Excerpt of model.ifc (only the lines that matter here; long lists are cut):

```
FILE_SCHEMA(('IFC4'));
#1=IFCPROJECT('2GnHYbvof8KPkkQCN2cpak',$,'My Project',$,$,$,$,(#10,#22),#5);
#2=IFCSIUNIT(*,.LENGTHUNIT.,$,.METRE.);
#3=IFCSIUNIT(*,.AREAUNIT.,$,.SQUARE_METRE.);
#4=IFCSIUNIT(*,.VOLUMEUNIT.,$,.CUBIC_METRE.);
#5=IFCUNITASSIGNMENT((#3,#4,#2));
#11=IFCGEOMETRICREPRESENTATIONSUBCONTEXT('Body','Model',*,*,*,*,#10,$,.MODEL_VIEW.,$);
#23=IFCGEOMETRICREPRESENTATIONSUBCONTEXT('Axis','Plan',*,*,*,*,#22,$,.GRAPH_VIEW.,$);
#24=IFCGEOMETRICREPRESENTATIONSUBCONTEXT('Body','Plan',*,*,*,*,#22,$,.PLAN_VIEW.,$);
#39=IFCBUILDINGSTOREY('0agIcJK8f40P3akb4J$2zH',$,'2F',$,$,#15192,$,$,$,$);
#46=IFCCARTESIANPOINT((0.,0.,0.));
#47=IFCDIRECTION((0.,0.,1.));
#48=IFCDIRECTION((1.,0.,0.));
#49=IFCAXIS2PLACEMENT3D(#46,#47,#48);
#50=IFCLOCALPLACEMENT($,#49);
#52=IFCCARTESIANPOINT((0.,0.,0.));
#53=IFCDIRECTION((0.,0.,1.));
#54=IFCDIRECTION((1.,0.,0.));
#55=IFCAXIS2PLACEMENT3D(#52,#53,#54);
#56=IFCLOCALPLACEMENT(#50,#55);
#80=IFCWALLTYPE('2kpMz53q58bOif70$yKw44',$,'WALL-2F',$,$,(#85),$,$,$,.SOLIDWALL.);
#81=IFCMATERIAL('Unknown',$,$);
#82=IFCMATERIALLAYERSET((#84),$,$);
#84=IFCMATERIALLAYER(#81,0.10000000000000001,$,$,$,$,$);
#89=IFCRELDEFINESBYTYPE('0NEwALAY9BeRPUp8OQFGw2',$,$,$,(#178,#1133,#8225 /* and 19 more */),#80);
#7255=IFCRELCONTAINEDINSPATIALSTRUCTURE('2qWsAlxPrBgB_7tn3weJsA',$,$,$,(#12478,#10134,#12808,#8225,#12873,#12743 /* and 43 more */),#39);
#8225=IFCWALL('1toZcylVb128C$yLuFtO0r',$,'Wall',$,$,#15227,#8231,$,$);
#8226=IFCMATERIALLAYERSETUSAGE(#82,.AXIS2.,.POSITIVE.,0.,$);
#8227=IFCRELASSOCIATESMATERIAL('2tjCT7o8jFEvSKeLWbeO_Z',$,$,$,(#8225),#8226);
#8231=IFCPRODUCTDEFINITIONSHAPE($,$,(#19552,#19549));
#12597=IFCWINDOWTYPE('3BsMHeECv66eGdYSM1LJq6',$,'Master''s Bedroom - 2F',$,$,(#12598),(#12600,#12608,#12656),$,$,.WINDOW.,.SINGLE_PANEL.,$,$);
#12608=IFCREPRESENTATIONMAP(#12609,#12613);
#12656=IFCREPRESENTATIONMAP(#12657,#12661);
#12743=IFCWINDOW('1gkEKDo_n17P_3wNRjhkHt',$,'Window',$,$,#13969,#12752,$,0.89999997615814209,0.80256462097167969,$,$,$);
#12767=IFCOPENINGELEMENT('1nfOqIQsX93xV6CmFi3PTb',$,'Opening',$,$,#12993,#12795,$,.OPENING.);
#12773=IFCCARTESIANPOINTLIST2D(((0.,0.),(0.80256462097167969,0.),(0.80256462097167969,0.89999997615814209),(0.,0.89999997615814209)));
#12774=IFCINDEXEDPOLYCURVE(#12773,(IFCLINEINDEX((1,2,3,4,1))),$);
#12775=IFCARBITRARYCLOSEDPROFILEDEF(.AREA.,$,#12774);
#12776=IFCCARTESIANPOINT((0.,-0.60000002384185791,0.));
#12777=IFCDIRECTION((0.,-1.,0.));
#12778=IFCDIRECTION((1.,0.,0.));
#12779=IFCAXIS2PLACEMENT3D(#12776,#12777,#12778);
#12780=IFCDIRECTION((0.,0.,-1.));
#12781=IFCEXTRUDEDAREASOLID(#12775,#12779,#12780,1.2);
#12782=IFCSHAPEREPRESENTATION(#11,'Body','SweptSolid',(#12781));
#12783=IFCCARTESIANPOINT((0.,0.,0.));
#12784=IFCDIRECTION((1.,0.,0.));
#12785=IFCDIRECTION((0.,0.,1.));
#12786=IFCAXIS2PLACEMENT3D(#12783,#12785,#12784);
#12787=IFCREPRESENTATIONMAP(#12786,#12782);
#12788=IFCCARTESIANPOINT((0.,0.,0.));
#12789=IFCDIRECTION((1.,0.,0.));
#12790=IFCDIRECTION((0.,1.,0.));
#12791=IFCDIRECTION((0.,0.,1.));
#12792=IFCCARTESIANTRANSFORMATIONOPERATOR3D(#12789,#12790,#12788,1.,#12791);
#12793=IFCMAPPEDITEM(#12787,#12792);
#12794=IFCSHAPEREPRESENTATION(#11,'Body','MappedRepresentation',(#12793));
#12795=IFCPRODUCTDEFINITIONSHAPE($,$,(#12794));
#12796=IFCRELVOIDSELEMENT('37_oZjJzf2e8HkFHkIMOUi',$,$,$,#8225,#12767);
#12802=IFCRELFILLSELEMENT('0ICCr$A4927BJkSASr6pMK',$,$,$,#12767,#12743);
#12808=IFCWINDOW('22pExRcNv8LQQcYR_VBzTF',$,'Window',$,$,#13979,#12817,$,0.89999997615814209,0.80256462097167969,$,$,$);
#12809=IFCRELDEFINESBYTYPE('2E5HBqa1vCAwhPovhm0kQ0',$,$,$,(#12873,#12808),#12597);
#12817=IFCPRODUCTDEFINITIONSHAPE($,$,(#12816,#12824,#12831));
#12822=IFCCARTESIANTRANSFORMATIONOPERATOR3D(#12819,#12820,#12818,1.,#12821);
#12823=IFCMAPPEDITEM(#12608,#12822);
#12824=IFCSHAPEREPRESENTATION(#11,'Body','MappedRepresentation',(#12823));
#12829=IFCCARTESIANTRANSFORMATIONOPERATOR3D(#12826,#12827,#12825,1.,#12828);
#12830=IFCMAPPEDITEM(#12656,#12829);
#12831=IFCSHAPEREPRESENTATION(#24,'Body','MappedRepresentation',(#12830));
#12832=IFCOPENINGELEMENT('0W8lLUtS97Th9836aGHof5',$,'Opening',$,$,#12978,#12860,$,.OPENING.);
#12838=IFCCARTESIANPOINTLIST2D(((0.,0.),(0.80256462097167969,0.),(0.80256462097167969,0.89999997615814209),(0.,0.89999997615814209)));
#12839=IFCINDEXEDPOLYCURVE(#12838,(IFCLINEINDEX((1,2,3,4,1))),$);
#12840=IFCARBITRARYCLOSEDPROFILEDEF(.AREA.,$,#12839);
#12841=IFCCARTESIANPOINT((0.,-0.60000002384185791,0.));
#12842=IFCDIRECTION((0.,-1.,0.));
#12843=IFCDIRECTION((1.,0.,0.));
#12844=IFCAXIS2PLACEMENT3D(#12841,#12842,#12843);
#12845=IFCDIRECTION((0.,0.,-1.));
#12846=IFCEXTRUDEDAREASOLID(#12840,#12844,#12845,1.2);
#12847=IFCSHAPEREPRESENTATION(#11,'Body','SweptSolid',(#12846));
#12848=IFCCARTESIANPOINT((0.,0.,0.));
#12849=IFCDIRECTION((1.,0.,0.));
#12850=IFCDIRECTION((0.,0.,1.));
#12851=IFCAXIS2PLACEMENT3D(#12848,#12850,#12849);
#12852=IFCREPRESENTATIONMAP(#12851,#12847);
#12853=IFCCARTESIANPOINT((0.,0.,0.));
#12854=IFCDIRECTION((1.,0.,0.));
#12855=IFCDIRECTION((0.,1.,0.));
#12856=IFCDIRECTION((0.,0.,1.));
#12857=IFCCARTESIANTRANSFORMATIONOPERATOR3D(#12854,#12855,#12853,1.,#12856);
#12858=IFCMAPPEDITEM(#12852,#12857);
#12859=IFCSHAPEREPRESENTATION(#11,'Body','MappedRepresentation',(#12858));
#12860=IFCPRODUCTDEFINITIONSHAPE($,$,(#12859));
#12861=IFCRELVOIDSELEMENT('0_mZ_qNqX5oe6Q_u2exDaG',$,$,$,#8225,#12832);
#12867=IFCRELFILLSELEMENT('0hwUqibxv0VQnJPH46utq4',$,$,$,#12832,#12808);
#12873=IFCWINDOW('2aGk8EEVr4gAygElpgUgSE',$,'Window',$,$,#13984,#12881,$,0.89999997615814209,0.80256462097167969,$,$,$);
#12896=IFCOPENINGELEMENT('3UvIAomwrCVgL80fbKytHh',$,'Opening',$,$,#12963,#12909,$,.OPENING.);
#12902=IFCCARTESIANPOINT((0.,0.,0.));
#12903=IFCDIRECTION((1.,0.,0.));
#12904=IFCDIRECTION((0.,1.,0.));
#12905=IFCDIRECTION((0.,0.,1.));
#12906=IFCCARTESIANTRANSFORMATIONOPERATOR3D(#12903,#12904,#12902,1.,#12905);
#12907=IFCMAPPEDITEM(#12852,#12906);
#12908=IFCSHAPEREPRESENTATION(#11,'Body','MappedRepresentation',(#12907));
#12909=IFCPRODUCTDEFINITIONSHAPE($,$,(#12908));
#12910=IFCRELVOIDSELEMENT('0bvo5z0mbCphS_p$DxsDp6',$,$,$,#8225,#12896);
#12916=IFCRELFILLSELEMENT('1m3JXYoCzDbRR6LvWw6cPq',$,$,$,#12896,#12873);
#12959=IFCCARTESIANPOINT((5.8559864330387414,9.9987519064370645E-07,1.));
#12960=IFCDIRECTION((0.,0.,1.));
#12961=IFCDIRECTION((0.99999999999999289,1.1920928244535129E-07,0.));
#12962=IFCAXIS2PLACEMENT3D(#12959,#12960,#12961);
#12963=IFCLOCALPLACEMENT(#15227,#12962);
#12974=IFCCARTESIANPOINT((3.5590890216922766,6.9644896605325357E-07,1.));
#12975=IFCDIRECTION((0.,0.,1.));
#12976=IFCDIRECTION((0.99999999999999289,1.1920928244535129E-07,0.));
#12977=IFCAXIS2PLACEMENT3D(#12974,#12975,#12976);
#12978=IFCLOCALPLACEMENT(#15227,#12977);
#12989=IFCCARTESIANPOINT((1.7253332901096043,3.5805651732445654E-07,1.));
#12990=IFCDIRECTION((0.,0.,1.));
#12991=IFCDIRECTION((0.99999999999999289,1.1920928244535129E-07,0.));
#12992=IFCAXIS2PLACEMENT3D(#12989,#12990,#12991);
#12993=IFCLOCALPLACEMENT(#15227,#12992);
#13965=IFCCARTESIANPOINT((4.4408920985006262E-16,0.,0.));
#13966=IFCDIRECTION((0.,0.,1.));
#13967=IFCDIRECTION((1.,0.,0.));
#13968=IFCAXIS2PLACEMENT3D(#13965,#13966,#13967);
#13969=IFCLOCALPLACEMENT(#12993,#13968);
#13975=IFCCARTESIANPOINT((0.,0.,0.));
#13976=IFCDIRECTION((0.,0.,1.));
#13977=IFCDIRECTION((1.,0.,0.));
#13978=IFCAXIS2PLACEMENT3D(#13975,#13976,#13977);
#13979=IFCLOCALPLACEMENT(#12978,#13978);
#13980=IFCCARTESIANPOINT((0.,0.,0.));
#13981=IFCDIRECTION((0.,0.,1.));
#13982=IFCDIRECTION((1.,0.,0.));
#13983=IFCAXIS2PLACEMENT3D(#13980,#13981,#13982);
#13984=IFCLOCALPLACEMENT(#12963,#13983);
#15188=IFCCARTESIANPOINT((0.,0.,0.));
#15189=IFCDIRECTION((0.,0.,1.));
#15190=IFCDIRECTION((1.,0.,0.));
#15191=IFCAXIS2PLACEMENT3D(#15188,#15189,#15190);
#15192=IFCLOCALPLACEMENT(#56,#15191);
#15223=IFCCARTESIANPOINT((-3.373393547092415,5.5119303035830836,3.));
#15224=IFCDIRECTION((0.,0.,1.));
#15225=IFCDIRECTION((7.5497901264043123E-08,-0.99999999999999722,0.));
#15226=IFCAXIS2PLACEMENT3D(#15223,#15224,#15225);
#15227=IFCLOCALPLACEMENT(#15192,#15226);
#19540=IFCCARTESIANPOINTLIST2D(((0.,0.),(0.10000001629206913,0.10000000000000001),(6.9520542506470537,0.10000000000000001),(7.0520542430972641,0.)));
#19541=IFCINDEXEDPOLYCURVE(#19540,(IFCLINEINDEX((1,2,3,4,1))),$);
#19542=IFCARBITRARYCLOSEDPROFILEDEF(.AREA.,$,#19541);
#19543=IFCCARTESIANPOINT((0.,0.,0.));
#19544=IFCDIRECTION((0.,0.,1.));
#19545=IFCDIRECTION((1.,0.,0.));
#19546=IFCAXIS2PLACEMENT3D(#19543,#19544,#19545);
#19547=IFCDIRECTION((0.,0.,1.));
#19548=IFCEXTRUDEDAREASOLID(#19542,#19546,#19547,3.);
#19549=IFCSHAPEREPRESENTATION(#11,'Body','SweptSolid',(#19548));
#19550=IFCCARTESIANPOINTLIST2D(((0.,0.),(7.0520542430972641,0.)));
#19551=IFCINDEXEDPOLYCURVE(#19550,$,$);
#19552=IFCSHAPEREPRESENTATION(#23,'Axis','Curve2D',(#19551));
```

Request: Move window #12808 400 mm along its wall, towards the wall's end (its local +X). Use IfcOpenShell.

```python
import ifcopenshell
import ifcopenshell.api.geometry
import ifcopenshell.util.placement

model = ifcopenshell.open("model.ifc")

window = model.by_guid("22pExRcNv8LQQcYR_VBzTF")
opening = window.FillsVoids[0].RelatingOpeningElement
wall = opening.VoidsElements[0].RelatingBuildingElement

wall_matrix = ifcopenshell.util.placement.get_local_placement(wall.ObjectPlacement)
shift = wall_matrix[:3, 0] * 0.4
before = ifcopenshell.util.placement.get_local_placement(window.ObjectPlacement)[:3, 3].copy()

# The window is placed relative to its opening, so it follows when the opening moves.
matrix = ifcopenshell.util.placement.get_local_placement(opening.ObjectPlacement)
matrix[:3, 3] += shift
ifcopenshell.api.geometry.edit_object_placement(
    model, product=opening, matrix=matrix, is_si=False, should_transform_children=True
)

after = ifcopenshell.util.placement.get_local_placement(window.ObjectPlacement)[:3, 3]
print("window moved by", (after - before).round(3) + 0.0)

model.write("model_edited.ifc")
```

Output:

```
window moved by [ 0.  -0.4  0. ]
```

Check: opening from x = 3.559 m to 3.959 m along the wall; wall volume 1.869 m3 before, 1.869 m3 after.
